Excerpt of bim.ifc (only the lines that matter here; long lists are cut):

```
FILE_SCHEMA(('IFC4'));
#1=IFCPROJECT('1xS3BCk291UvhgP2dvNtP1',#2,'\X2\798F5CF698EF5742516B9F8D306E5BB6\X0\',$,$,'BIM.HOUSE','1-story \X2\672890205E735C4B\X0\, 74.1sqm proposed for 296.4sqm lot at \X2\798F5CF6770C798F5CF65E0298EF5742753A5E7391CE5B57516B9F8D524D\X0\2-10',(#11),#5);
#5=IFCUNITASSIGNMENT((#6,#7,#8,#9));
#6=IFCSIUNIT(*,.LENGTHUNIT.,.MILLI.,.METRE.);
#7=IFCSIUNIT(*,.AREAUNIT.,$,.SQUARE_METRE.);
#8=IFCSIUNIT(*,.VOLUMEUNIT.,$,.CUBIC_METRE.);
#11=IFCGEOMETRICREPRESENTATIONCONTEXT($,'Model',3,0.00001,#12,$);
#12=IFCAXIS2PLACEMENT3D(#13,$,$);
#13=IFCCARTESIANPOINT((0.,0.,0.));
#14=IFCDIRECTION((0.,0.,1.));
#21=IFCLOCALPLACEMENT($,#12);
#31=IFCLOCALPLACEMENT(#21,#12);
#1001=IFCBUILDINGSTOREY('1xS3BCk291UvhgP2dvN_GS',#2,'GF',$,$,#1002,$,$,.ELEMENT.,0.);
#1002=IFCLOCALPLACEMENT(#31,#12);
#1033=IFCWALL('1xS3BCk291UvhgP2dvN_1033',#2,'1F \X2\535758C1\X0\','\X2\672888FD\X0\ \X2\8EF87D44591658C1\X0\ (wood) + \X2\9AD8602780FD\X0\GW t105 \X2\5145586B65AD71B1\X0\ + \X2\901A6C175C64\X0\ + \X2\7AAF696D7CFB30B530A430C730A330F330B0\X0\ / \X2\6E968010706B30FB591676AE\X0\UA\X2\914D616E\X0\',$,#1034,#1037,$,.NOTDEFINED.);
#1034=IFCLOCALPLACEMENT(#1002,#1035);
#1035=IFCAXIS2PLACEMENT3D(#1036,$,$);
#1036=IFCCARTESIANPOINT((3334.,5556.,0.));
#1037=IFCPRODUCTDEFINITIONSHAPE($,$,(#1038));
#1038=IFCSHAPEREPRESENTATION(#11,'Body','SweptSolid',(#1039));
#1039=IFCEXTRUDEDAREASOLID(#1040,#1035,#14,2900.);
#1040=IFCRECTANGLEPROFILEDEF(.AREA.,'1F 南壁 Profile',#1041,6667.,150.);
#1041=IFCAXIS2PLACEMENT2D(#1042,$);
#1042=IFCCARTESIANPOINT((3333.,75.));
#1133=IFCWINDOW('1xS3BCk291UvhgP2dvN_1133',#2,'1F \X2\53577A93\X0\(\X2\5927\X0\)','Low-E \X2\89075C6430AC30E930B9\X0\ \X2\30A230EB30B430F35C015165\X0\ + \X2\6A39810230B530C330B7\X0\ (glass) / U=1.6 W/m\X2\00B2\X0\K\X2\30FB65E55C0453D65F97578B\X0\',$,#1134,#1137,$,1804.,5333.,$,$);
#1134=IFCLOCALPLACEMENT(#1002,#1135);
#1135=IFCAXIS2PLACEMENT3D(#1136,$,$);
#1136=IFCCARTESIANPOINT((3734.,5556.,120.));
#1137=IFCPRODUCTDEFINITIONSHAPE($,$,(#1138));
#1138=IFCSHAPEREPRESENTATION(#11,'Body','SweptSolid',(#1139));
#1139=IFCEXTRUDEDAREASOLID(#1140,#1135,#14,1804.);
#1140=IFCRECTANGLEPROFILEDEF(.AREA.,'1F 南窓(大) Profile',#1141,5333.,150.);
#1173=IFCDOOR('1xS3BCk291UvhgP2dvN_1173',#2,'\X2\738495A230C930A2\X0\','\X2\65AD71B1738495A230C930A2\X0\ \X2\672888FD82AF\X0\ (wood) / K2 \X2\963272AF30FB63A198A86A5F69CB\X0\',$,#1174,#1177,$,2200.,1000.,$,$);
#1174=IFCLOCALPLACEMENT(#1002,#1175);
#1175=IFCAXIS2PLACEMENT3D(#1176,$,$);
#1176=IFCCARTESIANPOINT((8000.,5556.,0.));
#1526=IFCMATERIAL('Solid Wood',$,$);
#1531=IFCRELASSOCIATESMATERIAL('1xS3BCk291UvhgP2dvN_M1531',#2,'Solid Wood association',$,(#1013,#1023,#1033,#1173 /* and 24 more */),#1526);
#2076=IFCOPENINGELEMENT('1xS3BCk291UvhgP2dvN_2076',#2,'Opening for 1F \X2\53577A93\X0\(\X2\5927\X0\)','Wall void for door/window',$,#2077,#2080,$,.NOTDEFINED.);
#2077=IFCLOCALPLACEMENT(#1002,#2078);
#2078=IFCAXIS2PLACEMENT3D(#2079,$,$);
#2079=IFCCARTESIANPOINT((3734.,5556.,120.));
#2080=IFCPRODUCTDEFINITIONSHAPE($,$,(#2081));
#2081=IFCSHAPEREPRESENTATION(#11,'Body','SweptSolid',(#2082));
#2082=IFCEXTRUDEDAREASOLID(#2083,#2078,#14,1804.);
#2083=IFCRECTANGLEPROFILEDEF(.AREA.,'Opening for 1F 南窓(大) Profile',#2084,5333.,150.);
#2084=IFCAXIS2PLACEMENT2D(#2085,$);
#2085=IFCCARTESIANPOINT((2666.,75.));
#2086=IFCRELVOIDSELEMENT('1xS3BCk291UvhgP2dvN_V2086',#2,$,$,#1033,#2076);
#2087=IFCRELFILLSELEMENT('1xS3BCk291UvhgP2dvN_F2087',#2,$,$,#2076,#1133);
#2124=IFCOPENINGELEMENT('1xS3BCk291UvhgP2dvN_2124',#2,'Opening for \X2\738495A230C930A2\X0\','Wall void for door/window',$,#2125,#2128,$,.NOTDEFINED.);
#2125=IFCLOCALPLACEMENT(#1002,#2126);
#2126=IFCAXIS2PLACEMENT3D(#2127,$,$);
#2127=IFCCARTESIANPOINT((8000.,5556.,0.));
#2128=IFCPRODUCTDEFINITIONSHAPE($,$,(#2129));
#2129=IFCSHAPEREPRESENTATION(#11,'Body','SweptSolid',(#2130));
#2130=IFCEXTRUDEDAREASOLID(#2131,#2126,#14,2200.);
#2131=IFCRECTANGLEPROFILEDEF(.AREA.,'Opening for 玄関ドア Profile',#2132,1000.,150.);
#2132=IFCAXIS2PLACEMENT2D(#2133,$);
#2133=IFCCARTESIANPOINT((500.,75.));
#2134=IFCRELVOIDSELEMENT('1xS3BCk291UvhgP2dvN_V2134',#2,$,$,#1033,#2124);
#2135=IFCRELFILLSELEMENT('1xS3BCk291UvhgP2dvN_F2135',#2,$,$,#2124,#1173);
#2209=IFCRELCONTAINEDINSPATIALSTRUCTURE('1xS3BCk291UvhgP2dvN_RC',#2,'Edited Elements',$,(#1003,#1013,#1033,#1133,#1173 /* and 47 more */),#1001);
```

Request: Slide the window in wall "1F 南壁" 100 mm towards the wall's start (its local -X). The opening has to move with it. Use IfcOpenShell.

```python
import ifcopenshell
import ifcopenshell.api.geometry
import ifcopenshell.util.placement
import ifcopenshell.util.unit

model = ifcopenshell.open("bim.ifc")
unit_scale = ifcopenshell.util.unit.calculate_unit_scale(model)

window = model.by_id(1133)
opening = window.FillsVoids[0].RelatingOpeningElement
wall = opening.VoidsElements[0].RelatingBuildingElement

wall_matrix = ifcopenshell.util.placement.get_local_placement(wall.ObjectPlacement)
shift = wall_matrix[:3, 0] * -0.1 / unit_scale
before = ifcopenshell.util.placement.get_local_placement(window.ObjectPlacement)[:3, 3].copy()

# The window is not placed relative to its opening, so move both.
for product in (opening, window):
    matrix = ifcopenshell.util.placement.get_local_placement(product.ObjectPlacement)
    matrix[:3, 3] += shift
    ifcopenshell.api.geometry.edit_object_placement(model, product=product, matrix=matrix, is_si=False)

after = ifcopenshell.util.placement.get_local_placement(window.ObjectPlacement)[:3, 3]
print("window moved by", (after - before).round(3) + 0.0)

model.write("bim_edited.ifc")
```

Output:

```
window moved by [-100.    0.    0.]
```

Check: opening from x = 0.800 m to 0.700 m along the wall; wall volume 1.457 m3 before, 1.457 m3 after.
